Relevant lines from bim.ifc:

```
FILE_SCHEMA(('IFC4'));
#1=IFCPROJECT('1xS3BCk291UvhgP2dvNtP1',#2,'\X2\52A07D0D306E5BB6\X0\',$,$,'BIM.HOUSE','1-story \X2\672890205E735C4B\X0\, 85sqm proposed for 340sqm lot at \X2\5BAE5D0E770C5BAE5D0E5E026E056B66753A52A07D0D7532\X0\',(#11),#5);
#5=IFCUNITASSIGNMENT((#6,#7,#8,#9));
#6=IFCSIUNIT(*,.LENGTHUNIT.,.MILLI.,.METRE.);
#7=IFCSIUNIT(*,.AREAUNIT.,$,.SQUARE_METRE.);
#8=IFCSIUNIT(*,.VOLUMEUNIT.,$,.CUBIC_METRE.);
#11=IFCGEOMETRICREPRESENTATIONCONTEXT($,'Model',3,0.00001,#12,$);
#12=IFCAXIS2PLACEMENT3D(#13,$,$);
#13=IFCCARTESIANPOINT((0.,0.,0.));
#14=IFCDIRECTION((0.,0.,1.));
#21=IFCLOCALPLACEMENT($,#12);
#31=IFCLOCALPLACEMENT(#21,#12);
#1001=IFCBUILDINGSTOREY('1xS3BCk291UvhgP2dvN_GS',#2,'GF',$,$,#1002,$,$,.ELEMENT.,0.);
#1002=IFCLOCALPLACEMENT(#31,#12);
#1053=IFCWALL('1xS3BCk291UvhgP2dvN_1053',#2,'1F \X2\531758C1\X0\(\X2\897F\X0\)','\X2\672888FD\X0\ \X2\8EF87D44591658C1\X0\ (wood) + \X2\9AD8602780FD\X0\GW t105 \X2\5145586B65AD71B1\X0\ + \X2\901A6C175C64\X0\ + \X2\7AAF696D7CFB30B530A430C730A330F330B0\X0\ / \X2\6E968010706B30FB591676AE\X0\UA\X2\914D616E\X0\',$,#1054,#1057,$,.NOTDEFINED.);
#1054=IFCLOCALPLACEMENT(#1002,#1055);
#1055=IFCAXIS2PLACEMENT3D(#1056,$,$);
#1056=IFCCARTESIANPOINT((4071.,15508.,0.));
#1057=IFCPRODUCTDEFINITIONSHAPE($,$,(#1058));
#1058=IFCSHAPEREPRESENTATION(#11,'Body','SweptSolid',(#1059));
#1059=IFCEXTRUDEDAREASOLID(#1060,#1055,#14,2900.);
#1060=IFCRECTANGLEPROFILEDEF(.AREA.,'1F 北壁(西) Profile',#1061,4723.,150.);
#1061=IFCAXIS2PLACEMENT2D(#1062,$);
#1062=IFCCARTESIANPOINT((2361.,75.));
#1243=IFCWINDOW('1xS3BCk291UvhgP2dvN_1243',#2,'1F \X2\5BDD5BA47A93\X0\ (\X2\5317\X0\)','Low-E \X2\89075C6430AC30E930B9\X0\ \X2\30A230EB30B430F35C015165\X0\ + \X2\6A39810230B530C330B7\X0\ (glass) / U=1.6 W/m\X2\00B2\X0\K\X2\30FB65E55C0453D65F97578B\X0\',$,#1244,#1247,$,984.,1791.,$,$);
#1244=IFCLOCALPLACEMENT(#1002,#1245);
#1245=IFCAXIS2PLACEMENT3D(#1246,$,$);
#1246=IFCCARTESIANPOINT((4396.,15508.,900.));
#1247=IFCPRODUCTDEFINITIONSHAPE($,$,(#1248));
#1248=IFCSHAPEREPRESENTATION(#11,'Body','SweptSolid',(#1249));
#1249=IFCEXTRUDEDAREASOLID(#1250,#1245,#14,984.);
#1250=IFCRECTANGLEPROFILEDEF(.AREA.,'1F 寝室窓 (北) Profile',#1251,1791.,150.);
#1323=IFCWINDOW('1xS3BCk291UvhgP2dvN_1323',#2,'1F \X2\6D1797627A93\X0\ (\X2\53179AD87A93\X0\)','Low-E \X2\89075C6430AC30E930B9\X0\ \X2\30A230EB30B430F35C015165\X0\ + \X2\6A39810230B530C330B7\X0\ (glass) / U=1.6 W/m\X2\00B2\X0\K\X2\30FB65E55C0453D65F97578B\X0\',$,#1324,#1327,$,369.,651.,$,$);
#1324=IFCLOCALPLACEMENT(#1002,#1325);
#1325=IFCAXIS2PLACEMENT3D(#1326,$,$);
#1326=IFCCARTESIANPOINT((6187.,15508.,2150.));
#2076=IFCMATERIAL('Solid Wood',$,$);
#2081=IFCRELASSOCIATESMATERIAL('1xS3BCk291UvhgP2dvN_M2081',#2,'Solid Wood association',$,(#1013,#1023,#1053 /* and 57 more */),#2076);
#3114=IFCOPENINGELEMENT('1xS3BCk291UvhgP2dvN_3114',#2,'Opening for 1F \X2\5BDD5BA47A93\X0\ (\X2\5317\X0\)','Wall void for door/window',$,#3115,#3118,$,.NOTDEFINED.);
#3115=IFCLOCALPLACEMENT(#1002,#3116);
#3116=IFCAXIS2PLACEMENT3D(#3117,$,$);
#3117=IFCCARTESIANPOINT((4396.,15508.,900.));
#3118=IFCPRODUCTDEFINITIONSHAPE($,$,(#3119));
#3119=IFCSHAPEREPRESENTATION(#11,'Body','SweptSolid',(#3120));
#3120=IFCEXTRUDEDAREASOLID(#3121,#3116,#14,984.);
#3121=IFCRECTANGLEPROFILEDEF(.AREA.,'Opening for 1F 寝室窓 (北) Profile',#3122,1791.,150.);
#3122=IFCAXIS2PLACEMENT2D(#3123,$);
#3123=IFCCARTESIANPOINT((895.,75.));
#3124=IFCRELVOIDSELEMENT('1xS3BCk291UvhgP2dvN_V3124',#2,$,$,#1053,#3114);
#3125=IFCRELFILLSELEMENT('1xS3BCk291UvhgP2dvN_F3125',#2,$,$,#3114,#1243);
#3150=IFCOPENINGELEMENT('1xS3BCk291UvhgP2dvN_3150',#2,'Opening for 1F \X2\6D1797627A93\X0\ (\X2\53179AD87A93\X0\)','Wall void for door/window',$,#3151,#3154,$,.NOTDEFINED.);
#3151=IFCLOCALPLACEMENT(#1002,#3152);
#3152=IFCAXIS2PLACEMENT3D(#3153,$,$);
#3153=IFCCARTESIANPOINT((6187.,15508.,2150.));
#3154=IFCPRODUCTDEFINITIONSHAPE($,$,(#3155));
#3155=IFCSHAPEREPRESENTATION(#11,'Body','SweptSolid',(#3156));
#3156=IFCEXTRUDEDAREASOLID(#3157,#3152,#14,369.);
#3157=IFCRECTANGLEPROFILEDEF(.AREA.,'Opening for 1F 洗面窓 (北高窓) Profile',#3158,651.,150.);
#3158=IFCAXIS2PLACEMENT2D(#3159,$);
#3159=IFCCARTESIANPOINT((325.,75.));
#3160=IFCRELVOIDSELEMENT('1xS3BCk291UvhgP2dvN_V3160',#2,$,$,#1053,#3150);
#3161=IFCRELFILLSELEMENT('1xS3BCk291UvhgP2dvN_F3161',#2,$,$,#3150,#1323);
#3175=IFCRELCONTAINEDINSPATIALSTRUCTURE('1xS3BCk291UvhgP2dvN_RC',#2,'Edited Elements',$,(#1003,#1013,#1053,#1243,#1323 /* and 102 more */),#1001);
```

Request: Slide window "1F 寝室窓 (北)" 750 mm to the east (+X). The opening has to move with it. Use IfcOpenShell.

```python
import ifcopenshell
import ifcopenshell.api.geometry
import ifcopenshell.util.placement
import ifcopenshell.util.unit

model = ifcopenshell.open("bim.ifc")
unit_scale = ifcopenshell.util.unit.calculate_unit_scale(model)

window = model.by_guid("1xS3BCk291UvhgP2dvN_1243")
opening = window.FillsVoids[0].RelatingOpeningElement
wall = opening.VoidsElements[0].RelatingBuildingElement

wall_matrix = ifcopenshell.util.placement.get_local_placement(wall.ObjectPlacement)
shift = wall_matrix[:3, 0] * 0.75 / unit_scale
before = ifcopenshell.util.placement.get_local_placement(window.ObjectPlacement)[:3, 3].copy()

# The window is not placed relative to its opening, so move both.
for product in (opening, window):
    matrix = ifcopenshell.util.placement.get_local_placement(product.ObjectPlacement)
    matrix[:3, 3] += shift
    ifcopenshell.api.geometry.edit_object_placement(model, product=product, matrix=matrix, is_si=False)

after = ifcopenshell.util.placement.get_local_placement(window.ObjectPlacement)[:3, 3]
print("window moved by", (after - before).round(3) + 0.0)

model.write("bim_edited.ifc")
```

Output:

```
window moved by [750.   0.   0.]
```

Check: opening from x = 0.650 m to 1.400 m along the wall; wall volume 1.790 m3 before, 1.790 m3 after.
